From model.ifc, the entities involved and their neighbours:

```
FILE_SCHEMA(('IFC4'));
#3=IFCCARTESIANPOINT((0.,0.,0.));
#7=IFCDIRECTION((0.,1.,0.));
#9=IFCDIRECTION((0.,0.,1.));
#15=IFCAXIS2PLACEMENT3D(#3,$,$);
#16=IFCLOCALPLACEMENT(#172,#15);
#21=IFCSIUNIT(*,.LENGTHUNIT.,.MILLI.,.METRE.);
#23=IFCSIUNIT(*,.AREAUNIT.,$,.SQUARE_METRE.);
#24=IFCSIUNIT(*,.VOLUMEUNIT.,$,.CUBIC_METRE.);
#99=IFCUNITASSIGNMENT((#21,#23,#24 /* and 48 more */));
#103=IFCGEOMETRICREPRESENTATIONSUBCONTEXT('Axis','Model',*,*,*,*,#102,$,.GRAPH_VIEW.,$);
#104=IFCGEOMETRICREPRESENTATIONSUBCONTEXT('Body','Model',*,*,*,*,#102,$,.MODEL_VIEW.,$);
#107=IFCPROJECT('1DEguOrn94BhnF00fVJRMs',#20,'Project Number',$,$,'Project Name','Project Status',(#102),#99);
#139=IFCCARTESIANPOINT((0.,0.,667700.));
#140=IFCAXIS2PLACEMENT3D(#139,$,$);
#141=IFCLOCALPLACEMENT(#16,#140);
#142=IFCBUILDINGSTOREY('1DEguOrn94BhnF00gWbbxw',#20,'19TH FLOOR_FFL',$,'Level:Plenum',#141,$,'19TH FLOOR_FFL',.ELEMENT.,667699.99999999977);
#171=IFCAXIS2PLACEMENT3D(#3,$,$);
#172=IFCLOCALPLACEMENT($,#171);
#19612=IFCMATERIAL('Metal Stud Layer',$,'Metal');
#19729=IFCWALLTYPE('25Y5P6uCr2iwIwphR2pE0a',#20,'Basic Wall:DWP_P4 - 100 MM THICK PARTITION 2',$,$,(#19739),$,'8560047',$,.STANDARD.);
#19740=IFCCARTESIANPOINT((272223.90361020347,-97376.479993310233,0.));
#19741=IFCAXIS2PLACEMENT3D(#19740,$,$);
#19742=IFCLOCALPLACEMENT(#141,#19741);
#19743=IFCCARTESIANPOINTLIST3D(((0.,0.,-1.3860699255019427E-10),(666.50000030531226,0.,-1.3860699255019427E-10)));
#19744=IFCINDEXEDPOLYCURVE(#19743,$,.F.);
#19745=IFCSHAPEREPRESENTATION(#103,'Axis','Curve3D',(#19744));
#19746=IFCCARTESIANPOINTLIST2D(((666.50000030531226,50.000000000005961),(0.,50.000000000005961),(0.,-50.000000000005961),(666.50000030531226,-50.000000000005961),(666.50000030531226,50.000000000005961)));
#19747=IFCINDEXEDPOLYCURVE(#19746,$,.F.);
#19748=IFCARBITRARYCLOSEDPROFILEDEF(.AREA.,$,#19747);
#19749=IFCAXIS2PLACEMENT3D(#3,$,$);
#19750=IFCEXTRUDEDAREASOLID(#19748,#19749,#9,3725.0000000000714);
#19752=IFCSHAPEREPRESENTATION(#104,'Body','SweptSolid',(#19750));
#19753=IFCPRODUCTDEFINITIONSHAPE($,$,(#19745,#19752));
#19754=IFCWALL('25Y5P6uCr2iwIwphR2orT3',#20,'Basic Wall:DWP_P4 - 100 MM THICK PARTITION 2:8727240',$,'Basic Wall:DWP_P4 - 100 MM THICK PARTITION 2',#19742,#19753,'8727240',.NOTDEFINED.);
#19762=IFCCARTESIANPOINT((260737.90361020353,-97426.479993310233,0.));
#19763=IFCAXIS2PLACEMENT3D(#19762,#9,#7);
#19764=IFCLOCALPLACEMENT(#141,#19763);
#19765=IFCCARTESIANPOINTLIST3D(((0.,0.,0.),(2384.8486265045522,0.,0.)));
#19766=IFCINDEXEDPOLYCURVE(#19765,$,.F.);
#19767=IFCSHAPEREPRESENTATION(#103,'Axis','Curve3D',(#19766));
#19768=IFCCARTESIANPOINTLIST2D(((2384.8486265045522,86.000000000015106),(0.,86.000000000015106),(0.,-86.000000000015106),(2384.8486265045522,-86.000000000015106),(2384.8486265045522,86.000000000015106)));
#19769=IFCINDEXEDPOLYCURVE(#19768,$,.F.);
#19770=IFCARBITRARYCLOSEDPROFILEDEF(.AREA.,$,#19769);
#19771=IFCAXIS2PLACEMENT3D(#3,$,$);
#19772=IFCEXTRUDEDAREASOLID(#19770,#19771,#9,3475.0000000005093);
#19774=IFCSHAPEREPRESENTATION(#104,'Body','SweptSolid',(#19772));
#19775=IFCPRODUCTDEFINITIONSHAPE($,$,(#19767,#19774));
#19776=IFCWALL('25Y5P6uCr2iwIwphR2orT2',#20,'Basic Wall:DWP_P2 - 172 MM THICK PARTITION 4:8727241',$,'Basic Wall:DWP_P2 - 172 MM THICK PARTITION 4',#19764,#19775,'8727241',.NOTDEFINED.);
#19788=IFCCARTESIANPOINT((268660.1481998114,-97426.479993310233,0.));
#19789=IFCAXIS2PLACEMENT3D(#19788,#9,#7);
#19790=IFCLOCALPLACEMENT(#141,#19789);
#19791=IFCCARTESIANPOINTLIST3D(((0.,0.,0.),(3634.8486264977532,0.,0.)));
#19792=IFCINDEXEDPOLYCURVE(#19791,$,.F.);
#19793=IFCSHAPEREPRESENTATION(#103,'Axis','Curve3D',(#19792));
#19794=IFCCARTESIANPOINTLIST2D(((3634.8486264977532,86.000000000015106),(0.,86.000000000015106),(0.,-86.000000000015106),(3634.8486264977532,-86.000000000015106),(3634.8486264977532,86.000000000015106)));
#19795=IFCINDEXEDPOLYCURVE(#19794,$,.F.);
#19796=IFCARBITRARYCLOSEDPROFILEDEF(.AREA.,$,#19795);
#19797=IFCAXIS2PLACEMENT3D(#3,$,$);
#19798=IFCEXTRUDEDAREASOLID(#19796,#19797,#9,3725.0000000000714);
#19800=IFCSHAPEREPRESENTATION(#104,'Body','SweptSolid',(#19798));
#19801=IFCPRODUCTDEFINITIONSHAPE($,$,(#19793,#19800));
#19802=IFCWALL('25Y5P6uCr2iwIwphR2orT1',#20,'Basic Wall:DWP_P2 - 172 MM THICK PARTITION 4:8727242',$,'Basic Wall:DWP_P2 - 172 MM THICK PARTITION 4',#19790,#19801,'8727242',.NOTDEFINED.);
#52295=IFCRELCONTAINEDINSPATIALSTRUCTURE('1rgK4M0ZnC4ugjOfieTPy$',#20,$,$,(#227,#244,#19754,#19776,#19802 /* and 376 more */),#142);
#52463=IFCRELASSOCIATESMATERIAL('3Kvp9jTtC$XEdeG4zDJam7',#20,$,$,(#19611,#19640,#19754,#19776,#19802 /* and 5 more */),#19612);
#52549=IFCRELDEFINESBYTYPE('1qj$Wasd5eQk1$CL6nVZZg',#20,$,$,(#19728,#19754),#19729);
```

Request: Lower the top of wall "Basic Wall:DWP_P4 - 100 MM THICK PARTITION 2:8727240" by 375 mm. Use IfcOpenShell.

```python
import ifcopenshell
import ifcopenshell.geom
import ifcopenshell.util.representation
import ifcopenshell.util.shape

model = ifcopenshell.open("model.ifc")
settings = ifcopenshell.geom.settings()


def volume(element):
    """Net volume in cubic metres, openings subtracted."""
    shape = ifcopenshell.geom.create_shape(settings, element)
    return ifcopenshell.util.shape.get_volume(shape.geometry)


wall = model.by_guid("25Y5P6uCr2iwIwphR2orT3")
before = volume(wall)

body = ifcopenshell.util.representation.get_representation(wall, "Model", "Body")
solid = body.Items[0]
old_height = solid.Depth
solid.Depth -= 375.0
after = volume(wall)

print(f"height {old_height:g} -> {solid.Depth:g}, volume {before:.3f} -> {after:.3f} m3")

model.write("model-out.ifc")
```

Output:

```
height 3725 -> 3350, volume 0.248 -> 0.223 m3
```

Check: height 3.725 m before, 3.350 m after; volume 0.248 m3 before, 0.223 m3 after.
